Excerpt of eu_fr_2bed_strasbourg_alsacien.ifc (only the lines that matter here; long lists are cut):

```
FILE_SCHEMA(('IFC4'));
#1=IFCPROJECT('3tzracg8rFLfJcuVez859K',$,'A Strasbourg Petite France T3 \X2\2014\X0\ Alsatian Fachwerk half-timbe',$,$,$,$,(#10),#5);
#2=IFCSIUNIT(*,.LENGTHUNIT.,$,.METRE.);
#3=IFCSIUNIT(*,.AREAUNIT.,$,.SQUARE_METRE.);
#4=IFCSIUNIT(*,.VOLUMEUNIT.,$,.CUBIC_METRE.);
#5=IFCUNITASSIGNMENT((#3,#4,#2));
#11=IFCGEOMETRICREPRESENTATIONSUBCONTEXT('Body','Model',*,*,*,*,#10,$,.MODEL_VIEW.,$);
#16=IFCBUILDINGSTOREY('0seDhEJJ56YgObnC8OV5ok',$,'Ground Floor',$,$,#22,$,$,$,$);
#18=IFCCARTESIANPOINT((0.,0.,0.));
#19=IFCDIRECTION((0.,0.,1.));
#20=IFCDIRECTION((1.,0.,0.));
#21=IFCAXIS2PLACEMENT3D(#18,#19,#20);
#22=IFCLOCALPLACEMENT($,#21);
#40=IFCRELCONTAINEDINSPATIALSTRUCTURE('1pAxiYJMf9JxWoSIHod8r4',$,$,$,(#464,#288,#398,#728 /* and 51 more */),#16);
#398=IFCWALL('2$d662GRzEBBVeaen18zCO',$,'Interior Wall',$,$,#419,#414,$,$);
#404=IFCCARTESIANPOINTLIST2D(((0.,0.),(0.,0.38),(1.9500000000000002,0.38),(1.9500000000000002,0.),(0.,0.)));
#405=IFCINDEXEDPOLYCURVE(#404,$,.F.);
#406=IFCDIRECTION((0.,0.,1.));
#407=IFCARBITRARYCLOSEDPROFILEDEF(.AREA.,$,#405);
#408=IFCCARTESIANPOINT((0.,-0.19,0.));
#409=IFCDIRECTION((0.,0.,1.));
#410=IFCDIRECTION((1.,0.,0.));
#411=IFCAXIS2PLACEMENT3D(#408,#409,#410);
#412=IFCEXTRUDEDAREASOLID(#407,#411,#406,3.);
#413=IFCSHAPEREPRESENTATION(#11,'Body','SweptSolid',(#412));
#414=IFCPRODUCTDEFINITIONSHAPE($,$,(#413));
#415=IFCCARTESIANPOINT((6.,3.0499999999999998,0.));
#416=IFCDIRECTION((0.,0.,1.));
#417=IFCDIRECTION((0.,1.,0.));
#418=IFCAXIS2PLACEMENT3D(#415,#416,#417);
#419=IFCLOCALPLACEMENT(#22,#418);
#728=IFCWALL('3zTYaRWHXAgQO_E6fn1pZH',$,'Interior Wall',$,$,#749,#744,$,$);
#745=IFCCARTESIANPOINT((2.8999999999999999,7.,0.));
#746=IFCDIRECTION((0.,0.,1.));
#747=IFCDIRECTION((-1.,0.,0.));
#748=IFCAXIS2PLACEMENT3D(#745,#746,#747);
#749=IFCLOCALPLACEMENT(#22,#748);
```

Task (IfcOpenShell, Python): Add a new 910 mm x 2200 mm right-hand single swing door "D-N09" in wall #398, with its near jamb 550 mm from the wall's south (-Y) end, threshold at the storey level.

```python
import numpy as np
import ifcopenshell
import ifcopenshell.api.feature
import ifcopenshell.api.geometry
import ifcopenshell.api.root
import ifcopenshell.api.spatial
import ifcopenshell.geom
import ifcopenshell.util.element
import ifcopenshell.util.placement
import ifcopenshell.util.representation
import ifcopenshell.util.shape
import ifcopenshell.util.unit

model = ifcopenshell.open("eu_fr_2bed_strasbourg_alsacien.ifc")
unit_scale = ifcopenshell.util.unit.calculate_unit_scale(model)
settings = ifcopenshell.geom.settings()


def volume(element):
    """Net volume in cubic metres, openings subtracted."""
    shape = ifcopenshell.geom.create_shape(settings, element)
    return ifcopenshell.util.shape.get_volume(shape.geometry)


wall = model.by_id(398)
storey = ifcopenshell.util.element.get_container(wall, ifc_class="IfcBuildingStorey")
context = ifcopenshell.util.representation.get_context(model, "Model", "Body", "MODEL_VIEW")
before = volume(wall)

width, height, from_end, sill = 0.91, 2.2, 0.55, 0.0  # metres

# The wall runs along its own X axis, and the end named is its -X end.
wall_shape = ifcopenshell.geom.create_shape(settings, wall)
x, y, z = ifcopenshell.util.shape.get_vertices(wall_shape.geometry).T
start = x.min() + from_end
face, thickness = float(y.min()), float(y.max() - y.min())
wall_matrix = ifcopenshell.util.placement.get_local_placement(wall.ObjectPlacement)
level = ifcopenshell.util.placement.get_local_placement(storey.ObjectPlacement)[2, 3]


def in_wall(x, y):
    """Placement at x, y metres in the wall's axes, at sill height."""
    matrix = wall_matrix.copy()
    matrix[:, 3] = wall_matrix @ np.array([x / unit_scale, y / unit_scale, 0.0, 1.0])
    matrix[2, 3] = level + sill / unit_scale
    return matrix


# Opening: a box that overshoots both wall faces by 50 mm.
opening = ifcopenshell.api.root.create_entity(model, ifc_class="IfcOpeningElement", predefined_type="OPENING")
box = ifcopenshell.api.geometry.add_wall_representation(
    model, context=context, length=width, height=height, thickness=thickness + 0.1
)
ifcopenshell.api.geometry.assign_representation(model, product=opening, representation=box)
ifcopenshell.api.geometry.edit_object_placement(model, product=opening, matrix=in_wall(start, face - 0.05), is_si=False)
ifcopenshell.api.feature.add_feature(model, feature=opening, element=wall)

door = ifcopenshell.api.root.create_entity(model, ifc_class="IfcDoor", name="D-N09", predefined_type="DOOR")
door.OverallWidth, door.OverallHeight = width / unit_scale, height / unit_scale
door.OperationType = "SINGLE_SWING_RIGHT"
body = ifcopenshell.api.geometry.add_door_representation(
    model,
    context=context,
    overall_width=door.OverallWidth,
    overall_height=door.OverallHeight,
    operation_type="SINGLE_SWING_RIGHT",
    lining_properties={"LiningDepth": thickness / unit_scale, "ThresholdDepth": thickness / unit_scale},
)
ifcopenshell.api.geometry.assign_representation(model, product=door, representation=body)
ifcopenshell.api.spatial.assign_container(model, products=[door], relating_structure=storey)
ifcopenshell.api.feature.add_filling(model, opening=opening, element=door)

# The lining spans the wall, so the door starts at the wall face.
ifcopenshell.api.geometry.edit_object_placement(model, product=door, matrix=in_wall(start, face), is_si=False)

after = volume(wall)

print(f"wall volume {before:.3f} -> {after:.3f} m3")

model.write("eu_fr_2bed_strasbourg_alsacien_updated.ifc")
```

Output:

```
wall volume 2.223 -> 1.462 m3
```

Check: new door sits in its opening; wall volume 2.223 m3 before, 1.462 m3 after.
